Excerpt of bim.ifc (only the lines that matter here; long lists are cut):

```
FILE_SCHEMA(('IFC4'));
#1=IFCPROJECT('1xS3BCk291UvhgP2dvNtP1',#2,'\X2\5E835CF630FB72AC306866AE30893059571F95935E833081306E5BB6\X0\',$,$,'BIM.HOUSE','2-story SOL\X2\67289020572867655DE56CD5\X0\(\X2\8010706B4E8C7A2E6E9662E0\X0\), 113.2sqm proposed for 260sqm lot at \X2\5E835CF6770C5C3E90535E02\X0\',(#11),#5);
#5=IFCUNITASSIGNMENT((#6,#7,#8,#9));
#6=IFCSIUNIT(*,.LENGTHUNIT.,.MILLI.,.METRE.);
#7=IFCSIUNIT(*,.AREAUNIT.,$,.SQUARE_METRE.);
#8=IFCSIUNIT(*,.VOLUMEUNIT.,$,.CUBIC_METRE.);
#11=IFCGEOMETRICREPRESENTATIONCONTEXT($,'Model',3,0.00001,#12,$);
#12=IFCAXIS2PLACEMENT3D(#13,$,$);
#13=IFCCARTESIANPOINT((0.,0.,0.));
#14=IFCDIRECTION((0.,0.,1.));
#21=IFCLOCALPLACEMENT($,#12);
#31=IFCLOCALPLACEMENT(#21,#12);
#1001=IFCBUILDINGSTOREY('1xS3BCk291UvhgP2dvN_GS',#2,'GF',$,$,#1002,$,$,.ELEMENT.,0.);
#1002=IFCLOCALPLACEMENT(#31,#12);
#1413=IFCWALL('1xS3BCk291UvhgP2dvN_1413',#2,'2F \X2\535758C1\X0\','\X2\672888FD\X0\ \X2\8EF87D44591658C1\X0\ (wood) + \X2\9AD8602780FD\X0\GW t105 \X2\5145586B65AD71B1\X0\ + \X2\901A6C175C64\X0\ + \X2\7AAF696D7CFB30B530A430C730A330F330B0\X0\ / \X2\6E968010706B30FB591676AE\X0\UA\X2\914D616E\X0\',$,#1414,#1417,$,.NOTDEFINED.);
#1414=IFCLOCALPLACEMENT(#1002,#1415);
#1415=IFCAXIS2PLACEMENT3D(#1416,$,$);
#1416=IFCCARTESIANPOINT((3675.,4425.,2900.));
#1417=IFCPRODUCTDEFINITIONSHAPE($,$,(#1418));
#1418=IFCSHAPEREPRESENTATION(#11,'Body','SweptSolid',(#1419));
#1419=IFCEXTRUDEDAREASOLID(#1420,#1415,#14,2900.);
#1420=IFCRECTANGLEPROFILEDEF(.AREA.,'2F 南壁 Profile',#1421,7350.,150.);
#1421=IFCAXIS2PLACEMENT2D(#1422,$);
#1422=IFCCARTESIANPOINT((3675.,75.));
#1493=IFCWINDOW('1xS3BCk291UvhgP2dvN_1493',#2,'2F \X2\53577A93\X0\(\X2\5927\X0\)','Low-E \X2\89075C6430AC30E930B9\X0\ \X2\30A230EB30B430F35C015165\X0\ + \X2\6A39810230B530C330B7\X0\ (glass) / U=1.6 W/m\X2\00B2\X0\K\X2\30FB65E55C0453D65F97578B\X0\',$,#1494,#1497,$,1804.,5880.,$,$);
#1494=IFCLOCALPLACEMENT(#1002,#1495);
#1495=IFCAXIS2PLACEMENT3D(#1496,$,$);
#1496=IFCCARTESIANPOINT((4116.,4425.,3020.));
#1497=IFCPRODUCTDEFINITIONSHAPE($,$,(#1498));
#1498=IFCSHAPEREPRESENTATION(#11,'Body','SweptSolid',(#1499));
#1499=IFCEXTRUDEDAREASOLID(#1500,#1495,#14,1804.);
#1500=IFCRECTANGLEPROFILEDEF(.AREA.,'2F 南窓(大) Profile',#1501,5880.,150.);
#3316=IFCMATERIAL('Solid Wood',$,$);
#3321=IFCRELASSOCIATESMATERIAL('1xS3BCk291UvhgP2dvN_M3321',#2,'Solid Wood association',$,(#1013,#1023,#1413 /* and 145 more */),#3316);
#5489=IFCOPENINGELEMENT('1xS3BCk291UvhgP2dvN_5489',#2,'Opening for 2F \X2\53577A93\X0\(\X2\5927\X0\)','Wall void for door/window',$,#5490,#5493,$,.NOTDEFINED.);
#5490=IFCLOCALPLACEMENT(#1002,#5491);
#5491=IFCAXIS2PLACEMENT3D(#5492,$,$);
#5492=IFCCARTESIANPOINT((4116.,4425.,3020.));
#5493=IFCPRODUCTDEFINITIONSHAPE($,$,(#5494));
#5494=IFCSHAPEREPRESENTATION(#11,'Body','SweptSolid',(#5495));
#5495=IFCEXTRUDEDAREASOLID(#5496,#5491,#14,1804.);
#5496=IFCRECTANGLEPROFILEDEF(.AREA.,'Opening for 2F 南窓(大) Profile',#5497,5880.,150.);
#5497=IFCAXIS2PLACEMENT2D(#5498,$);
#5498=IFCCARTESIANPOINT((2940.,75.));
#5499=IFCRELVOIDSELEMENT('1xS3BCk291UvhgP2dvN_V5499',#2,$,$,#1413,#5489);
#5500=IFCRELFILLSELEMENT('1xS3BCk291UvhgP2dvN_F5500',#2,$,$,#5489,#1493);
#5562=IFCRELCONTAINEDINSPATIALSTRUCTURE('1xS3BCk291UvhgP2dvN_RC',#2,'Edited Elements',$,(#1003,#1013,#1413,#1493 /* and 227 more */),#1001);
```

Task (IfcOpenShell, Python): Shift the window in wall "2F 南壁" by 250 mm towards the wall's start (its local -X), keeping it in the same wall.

```python
import ifcopenshell
import ifcopenshell.api.geometry
import ifcopenshell.util.placement
import ifcopenshell.util.unit

model = ifcopenshell.open("bim.ifc")
unit_scale = ifcopenshell.util.unit.calculate_unit_scale(model)

window = model.by_guid("1xS3BCk291UvhgP2dvN_1493")
opening = window.FillsVoids[0].RelatingOpeningElement
wall = opening.VoidsElements[0].RelatingBuildingElement

wall_matrix = ifcopenshell.util.placement.get_local_placement(wall.ObjectPlacement)
shift = wall_matrix[:3, 0] * -0.25 / unit_scale
before = ifcopenshell.util.placement.get_local_placement(window.ObjectPlacement)[:3, 3].copy()

# The window is not placed relative to its opening, so move both.
for product in (opening, window):
    matrix = ifcopenshell.util.placement.get_local_placement(product.ObjectPlacement)
    matrix[:3, 3] += shift
    ifcopenshell.api.geometry.edit_object_placement(model, product=product, matrix=matrix, is_si=False)

after = ifcopenshell.util.placement.get_local_placement(window.ObjectPlacement)[:3, 3]
print("window moved by", (after - before).round(3) + 0.0)

model.write("bim_updated.ifc")
```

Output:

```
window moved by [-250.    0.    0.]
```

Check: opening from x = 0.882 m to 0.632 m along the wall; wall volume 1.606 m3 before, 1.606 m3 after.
